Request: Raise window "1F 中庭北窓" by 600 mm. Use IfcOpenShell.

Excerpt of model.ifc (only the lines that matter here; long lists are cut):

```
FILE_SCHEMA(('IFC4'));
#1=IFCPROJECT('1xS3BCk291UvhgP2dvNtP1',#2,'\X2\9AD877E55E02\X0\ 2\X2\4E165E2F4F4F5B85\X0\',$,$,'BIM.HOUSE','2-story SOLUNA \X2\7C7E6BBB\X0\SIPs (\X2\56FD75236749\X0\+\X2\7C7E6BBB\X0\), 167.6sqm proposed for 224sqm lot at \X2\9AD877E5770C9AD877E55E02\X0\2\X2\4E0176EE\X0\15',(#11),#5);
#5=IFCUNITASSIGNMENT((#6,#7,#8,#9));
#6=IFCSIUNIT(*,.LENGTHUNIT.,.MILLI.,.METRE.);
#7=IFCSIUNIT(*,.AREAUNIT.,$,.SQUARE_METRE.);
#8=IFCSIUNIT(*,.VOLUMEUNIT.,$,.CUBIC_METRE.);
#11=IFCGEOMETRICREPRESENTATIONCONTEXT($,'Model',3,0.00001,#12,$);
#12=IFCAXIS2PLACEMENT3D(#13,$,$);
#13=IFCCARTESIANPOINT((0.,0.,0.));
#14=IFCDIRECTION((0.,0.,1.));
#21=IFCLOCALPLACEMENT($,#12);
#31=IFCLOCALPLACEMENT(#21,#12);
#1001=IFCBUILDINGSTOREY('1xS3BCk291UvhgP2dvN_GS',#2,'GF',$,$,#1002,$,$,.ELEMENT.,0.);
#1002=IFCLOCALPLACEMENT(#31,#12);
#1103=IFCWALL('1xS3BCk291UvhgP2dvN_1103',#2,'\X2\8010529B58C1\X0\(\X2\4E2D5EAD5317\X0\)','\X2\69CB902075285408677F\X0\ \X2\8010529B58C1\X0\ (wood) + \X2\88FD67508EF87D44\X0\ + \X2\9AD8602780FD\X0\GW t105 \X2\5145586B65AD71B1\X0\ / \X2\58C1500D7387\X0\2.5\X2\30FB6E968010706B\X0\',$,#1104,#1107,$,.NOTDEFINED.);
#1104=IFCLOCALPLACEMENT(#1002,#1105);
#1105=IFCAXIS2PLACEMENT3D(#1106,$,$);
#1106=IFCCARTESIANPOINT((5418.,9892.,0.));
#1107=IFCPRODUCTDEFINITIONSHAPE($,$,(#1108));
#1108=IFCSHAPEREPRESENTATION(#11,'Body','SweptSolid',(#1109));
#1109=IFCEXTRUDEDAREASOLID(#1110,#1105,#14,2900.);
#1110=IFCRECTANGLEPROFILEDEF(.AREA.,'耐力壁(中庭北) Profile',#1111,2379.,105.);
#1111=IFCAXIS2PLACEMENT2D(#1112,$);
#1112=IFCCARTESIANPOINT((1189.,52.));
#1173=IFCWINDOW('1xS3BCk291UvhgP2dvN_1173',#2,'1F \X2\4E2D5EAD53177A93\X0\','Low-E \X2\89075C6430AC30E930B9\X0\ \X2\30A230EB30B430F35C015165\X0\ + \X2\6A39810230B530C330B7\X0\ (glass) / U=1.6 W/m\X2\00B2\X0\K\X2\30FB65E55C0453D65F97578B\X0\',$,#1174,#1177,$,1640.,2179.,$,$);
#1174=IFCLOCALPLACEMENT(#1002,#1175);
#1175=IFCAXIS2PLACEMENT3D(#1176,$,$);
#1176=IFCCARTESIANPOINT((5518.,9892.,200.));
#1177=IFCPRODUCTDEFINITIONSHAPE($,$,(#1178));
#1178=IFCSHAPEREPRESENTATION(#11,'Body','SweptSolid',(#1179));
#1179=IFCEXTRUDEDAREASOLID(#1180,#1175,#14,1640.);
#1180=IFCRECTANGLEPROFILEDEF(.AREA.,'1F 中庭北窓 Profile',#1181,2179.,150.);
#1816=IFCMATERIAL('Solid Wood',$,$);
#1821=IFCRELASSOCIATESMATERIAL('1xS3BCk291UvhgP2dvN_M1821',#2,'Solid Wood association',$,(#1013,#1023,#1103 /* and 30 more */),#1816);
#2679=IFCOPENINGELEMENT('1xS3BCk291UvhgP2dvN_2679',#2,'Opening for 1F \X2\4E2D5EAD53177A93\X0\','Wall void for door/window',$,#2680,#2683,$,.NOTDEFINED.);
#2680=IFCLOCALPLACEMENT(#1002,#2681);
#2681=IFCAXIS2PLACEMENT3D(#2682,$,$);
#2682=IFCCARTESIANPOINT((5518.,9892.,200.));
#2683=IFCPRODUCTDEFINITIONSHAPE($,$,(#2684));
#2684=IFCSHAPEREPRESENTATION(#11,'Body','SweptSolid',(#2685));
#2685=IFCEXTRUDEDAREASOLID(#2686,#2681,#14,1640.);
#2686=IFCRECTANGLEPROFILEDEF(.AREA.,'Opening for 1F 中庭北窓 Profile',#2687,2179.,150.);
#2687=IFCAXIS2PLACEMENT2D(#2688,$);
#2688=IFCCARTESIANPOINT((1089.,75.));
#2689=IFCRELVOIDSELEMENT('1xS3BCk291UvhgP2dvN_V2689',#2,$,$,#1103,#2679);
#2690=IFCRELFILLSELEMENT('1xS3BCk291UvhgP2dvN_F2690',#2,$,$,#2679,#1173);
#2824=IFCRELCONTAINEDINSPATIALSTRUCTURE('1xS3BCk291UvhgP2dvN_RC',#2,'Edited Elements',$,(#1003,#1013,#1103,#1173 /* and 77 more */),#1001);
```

```python
import numpy as np
import ifcopenshell
import ifcopenshell.api.geometry
import ifcopenshell.util.placement
import ifcopenshell.util.unit

model = ifcopenshell.open("model.ifc")
unit_scale = ifcopenshell.util.unit.calculate_unit_scale(model)

window = model.by_guid("1xS3BCk291UvhgP2dvN_1173")
opening = window.FillsVoids[0].RelatingOpeningElement
dz = 0.6 / unit_scale

shift = np.array([0.0, 0.0, dz])
# The window is not placed relative to its opening, so move both.
for product in (opening, window):
    matrix = ifcopenshell.util.placement.get_local_placement(product.ObjectPlacement)
    matrix[:3, 3] += shift
    ifcopenshell.api.geometry.edit_object_placement(model, product=product, matrix=matrix, is_si=False)

print(f"moved by {dz * unit_scale:+.3f} m")

model.write("model-out.ifc")
```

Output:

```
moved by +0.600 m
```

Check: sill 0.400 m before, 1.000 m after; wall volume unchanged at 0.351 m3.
